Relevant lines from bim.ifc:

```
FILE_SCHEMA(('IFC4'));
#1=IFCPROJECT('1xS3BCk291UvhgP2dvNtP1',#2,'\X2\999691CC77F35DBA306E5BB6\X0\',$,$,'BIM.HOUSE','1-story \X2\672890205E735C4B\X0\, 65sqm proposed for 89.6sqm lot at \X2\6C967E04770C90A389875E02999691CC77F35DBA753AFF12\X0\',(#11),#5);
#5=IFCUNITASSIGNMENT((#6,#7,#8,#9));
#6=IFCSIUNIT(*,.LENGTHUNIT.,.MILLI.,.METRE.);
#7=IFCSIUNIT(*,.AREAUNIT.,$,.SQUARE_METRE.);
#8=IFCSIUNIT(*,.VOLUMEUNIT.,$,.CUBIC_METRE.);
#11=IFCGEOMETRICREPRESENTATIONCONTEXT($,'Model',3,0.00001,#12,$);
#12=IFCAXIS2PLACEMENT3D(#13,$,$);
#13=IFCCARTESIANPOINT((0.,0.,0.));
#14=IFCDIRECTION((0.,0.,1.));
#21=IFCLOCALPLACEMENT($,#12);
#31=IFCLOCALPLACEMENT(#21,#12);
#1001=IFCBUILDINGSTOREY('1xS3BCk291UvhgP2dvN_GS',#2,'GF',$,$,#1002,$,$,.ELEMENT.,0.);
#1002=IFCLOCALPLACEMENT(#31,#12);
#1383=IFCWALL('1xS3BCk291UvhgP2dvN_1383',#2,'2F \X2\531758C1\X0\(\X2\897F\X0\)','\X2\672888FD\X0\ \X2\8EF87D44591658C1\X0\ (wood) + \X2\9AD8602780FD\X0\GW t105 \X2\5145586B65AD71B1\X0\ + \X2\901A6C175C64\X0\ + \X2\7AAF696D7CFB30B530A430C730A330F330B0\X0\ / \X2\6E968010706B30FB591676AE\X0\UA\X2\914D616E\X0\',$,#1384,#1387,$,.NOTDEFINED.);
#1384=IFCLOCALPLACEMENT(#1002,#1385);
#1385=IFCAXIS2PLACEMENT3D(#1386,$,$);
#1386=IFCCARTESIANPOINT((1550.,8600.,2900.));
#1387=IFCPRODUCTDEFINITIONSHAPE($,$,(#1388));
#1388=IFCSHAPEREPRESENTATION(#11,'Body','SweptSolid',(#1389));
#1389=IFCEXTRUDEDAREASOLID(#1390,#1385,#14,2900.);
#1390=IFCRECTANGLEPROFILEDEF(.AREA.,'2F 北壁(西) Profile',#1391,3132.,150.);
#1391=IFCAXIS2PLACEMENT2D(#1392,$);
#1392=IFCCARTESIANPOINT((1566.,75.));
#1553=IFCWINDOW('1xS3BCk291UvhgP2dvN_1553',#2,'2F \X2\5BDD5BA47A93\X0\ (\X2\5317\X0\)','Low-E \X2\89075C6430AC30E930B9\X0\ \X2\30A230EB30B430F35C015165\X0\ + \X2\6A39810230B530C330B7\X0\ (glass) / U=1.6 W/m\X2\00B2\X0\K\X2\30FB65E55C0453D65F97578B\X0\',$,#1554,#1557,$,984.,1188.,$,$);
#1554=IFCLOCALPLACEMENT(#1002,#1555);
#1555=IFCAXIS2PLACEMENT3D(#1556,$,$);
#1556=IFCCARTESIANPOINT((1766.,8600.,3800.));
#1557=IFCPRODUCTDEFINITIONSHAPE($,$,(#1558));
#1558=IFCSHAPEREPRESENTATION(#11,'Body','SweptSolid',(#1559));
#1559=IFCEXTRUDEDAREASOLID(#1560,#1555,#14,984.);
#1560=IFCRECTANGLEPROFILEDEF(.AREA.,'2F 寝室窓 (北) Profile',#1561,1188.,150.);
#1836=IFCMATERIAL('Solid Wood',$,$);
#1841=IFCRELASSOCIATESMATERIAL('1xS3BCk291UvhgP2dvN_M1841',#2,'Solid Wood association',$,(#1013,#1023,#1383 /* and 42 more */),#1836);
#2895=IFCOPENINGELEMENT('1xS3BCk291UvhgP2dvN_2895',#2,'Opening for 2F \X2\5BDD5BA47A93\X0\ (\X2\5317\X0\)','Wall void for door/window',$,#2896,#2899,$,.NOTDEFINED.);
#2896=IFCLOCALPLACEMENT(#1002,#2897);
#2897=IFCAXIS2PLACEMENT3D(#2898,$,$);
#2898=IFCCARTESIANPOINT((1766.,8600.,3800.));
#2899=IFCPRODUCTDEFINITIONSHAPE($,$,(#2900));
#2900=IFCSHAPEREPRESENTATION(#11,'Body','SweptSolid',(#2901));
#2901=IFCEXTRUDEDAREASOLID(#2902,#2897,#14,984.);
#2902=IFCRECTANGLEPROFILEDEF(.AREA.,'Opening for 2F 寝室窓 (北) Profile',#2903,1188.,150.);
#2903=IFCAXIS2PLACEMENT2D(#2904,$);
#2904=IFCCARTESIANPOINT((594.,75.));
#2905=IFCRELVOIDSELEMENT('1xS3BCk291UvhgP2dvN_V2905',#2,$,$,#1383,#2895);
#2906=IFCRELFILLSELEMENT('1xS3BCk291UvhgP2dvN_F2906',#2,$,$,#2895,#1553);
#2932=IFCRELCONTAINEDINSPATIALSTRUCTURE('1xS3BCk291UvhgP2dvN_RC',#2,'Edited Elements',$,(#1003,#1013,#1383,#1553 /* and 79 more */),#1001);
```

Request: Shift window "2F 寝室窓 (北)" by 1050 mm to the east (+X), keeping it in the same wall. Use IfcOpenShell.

```python
import ifcopenshell
import ifcopenshell.api.geometry
import ifcopenshell.util.placement
import ifcopenshell.util.unit

model = ifcopenshell.open("bim.ifc")
unit_scale = ifcopenshell.util.unit.calculate_unit_scale(model)

window = model.by_guid("1xS3BCk291UvhgP2dvN_1553")
opening = window.FillsVoids[0].RelatingOpeningElement
wall = opening.VoidsElements[0].RelatingBuildingElement

wall_matrix = ifcopenshell.util.placement.get_local_placement(wall.ObjectPlacement)
shift = wall_matrix[:3, 0] * 1.05 / unit_scale
before = ifcopenshell.util.placement.get_local_placement(window.ObjectPlacement)[:3, 3].copy()

# The window is not placed relative to its opening, so move both.
for product in (opening, window):
    matrix = ifcopenshell.util.placement.get_local_placement(product.ObjectPlacement)
    matrix[:3, 3] += shift
    ifcopenshell.api.geometry.edit_object_placement(model, product=product, matrix=matrix, is_si=False)

after = ifcopenshell.util.placement.get_local_placement(window.ObjectPlacement)[:3, 3]
print("window moved by", (after - before).round(3) + 0.0)

model.write("bim_v2.ifc")
```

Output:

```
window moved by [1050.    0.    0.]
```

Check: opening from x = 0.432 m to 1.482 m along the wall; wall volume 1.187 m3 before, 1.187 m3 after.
